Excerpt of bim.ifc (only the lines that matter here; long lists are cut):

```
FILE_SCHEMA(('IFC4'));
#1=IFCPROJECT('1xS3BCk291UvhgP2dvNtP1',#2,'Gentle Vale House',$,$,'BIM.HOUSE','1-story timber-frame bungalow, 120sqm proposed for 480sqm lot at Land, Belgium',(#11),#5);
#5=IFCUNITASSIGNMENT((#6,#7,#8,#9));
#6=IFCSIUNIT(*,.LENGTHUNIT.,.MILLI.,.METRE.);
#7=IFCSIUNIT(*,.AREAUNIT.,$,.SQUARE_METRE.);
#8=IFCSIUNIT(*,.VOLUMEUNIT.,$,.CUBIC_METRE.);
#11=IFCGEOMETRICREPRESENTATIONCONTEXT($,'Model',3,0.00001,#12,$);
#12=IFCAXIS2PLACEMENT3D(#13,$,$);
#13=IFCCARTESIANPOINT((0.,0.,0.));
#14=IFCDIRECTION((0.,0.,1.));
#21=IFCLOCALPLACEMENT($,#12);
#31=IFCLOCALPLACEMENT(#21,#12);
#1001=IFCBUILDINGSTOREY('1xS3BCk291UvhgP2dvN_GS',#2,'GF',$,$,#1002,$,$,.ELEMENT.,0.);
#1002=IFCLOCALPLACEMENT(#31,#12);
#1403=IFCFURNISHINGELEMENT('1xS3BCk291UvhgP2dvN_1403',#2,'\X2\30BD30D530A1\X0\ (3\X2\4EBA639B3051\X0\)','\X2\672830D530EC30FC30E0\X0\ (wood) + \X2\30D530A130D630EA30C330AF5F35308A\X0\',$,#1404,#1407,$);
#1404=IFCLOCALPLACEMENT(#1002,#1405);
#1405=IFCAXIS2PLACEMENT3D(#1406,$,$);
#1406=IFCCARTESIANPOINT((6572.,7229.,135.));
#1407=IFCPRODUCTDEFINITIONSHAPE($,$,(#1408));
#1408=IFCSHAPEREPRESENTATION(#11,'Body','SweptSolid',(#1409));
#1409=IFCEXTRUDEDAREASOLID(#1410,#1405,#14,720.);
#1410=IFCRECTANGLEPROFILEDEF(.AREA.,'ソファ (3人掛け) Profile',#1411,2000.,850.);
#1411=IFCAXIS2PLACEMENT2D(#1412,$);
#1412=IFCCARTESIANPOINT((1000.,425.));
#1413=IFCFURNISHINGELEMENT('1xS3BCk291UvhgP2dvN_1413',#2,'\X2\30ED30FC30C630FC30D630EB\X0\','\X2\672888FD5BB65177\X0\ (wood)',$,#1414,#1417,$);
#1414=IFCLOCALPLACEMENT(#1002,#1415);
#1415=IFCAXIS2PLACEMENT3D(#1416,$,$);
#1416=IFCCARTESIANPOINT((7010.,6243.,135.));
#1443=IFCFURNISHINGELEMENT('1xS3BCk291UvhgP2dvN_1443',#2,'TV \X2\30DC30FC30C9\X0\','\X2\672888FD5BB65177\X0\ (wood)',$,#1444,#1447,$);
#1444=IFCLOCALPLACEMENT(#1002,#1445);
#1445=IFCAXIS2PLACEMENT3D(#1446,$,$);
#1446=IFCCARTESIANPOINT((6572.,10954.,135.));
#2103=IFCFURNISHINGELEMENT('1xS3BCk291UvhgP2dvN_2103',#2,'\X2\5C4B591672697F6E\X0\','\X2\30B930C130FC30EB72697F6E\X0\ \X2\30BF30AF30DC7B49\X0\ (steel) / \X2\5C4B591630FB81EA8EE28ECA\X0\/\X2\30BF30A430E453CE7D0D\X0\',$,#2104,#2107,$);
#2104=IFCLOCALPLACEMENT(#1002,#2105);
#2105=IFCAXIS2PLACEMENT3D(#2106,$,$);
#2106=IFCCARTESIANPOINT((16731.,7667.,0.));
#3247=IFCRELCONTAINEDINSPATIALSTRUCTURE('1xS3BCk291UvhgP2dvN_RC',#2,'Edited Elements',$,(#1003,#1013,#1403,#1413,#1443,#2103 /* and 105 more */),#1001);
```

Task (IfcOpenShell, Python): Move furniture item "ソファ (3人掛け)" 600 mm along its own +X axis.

```python
import ifcopenshell
import ifcopenshell.api.geometry
import ifcopenshell.util.placement
import ifcopenshell.util.unit

model = ifcopenshell.open("bim.ifc")
unit_scale = ifcopenshell.util.unit.calculate_unit_scale(model)

item = model.by_guid("1xS3BCk291UvhgP2dvN_1403")
matrix = ifcopenshell.util.placement.get_local_placement(item.ObjectPlacement)
matrix[:3, 3] += matrix[:3, 0] * 0.6 / unit_scale
ifcopenshell.api.geometry.edit_object_placement(model, product=item, matrix=matrix, is_si=False)

print(ifcopenshell.util.placement.get_local_placement(item.ObjectPlacement).round(3) + 0.0)

model.write("bim_edited.ifc")
```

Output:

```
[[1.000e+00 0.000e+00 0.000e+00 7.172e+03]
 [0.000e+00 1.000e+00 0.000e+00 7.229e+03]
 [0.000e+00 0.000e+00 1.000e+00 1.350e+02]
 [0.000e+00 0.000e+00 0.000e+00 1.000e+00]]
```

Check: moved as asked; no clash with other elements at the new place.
